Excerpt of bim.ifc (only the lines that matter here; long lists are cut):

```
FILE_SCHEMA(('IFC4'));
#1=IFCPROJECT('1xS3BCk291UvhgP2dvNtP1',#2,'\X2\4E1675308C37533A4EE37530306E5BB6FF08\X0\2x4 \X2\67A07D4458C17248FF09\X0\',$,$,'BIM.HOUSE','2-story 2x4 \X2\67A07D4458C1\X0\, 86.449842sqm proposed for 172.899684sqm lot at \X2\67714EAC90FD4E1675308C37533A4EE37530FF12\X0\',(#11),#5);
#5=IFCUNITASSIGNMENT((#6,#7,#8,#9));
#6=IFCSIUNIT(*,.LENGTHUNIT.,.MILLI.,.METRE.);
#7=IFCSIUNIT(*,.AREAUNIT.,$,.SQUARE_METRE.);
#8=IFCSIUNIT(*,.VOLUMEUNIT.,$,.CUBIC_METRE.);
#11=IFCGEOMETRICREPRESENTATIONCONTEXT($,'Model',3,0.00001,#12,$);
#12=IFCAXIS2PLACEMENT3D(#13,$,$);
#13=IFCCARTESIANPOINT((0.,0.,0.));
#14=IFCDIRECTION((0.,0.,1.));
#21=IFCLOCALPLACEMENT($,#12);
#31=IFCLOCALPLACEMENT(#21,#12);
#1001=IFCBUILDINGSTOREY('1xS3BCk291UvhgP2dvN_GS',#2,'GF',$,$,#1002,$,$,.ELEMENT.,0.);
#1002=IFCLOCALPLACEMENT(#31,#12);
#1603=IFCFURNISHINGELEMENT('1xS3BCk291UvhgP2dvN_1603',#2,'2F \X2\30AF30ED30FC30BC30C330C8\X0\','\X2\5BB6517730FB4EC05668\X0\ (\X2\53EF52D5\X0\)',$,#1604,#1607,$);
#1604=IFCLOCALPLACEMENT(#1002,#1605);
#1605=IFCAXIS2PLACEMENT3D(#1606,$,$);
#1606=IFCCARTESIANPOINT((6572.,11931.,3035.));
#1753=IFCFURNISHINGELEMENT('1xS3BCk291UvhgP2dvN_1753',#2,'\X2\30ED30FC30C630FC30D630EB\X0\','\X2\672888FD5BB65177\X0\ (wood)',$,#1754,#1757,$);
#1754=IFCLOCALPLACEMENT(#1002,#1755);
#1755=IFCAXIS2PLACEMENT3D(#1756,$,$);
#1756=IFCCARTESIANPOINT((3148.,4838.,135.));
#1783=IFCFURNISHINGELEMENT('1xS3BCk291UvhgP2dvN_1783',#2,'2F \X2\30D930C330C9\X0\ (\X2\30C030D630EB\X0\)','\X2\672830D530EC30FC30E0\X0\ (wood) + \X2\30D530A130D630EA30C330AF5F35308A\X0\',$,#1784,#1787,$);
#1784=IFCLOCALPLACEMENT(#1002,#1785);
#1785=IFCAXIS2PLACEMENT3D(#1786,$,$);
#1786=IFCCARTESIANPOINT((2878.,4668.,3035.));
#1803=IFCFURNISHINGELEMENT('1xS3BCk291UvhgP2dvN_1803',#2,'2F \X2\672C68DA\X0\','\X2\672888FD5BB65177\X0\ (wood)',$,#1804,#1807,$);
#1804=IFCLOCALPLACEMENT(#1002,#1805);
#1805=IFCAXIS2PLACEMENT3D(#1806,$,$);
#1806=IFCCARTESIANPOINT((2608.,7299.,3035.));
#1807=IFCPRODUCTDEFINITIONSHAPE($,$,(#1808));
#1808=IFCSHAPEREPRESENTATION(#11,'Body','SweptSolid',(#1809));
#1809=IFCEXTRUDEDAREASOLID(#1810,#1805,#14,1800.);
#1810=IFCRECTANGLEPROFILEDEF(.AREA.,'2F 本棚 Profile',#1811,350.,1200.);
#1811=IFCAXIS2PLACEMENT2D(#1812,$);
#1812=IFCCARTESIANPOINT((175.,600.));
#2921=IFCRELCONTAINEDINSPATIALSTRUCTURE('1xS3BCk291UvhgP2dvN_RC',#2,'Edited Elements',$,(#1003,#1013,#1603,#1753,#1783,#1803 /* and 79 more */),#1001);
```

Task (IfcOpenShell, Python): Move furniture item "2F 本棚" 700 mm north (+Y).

```python
import ifcopenshell
import ifcopenshell.api.geometry
import ifcopenshell.util.placement

model = ifcopenshell.open("bim.ifc")

item = model.by_guid("1xS3BCk291UvhgP2dvN_1803")
matrix = ifcopenshell.util.placement.get_local_placement(item.ObjectPlacement)
matrix[1, 3] += 700.0
ifcopenshell.api.geometry.edit_object_placement(model, product=item, matrix=matrix, is_si=False)

print(ifcopenshell.util.placement.get_local_placement(item.ObjectPlacement).round(3) + 0.0)

model.write("bim-out.ifc")
```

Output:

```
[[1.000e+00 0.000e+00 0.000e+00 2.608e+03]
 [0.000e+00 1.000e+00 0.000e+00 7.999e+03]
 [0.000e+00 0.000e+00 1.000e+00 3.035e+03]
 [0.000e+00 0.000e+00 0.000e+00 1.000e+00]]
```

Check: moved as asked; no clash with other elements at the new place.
